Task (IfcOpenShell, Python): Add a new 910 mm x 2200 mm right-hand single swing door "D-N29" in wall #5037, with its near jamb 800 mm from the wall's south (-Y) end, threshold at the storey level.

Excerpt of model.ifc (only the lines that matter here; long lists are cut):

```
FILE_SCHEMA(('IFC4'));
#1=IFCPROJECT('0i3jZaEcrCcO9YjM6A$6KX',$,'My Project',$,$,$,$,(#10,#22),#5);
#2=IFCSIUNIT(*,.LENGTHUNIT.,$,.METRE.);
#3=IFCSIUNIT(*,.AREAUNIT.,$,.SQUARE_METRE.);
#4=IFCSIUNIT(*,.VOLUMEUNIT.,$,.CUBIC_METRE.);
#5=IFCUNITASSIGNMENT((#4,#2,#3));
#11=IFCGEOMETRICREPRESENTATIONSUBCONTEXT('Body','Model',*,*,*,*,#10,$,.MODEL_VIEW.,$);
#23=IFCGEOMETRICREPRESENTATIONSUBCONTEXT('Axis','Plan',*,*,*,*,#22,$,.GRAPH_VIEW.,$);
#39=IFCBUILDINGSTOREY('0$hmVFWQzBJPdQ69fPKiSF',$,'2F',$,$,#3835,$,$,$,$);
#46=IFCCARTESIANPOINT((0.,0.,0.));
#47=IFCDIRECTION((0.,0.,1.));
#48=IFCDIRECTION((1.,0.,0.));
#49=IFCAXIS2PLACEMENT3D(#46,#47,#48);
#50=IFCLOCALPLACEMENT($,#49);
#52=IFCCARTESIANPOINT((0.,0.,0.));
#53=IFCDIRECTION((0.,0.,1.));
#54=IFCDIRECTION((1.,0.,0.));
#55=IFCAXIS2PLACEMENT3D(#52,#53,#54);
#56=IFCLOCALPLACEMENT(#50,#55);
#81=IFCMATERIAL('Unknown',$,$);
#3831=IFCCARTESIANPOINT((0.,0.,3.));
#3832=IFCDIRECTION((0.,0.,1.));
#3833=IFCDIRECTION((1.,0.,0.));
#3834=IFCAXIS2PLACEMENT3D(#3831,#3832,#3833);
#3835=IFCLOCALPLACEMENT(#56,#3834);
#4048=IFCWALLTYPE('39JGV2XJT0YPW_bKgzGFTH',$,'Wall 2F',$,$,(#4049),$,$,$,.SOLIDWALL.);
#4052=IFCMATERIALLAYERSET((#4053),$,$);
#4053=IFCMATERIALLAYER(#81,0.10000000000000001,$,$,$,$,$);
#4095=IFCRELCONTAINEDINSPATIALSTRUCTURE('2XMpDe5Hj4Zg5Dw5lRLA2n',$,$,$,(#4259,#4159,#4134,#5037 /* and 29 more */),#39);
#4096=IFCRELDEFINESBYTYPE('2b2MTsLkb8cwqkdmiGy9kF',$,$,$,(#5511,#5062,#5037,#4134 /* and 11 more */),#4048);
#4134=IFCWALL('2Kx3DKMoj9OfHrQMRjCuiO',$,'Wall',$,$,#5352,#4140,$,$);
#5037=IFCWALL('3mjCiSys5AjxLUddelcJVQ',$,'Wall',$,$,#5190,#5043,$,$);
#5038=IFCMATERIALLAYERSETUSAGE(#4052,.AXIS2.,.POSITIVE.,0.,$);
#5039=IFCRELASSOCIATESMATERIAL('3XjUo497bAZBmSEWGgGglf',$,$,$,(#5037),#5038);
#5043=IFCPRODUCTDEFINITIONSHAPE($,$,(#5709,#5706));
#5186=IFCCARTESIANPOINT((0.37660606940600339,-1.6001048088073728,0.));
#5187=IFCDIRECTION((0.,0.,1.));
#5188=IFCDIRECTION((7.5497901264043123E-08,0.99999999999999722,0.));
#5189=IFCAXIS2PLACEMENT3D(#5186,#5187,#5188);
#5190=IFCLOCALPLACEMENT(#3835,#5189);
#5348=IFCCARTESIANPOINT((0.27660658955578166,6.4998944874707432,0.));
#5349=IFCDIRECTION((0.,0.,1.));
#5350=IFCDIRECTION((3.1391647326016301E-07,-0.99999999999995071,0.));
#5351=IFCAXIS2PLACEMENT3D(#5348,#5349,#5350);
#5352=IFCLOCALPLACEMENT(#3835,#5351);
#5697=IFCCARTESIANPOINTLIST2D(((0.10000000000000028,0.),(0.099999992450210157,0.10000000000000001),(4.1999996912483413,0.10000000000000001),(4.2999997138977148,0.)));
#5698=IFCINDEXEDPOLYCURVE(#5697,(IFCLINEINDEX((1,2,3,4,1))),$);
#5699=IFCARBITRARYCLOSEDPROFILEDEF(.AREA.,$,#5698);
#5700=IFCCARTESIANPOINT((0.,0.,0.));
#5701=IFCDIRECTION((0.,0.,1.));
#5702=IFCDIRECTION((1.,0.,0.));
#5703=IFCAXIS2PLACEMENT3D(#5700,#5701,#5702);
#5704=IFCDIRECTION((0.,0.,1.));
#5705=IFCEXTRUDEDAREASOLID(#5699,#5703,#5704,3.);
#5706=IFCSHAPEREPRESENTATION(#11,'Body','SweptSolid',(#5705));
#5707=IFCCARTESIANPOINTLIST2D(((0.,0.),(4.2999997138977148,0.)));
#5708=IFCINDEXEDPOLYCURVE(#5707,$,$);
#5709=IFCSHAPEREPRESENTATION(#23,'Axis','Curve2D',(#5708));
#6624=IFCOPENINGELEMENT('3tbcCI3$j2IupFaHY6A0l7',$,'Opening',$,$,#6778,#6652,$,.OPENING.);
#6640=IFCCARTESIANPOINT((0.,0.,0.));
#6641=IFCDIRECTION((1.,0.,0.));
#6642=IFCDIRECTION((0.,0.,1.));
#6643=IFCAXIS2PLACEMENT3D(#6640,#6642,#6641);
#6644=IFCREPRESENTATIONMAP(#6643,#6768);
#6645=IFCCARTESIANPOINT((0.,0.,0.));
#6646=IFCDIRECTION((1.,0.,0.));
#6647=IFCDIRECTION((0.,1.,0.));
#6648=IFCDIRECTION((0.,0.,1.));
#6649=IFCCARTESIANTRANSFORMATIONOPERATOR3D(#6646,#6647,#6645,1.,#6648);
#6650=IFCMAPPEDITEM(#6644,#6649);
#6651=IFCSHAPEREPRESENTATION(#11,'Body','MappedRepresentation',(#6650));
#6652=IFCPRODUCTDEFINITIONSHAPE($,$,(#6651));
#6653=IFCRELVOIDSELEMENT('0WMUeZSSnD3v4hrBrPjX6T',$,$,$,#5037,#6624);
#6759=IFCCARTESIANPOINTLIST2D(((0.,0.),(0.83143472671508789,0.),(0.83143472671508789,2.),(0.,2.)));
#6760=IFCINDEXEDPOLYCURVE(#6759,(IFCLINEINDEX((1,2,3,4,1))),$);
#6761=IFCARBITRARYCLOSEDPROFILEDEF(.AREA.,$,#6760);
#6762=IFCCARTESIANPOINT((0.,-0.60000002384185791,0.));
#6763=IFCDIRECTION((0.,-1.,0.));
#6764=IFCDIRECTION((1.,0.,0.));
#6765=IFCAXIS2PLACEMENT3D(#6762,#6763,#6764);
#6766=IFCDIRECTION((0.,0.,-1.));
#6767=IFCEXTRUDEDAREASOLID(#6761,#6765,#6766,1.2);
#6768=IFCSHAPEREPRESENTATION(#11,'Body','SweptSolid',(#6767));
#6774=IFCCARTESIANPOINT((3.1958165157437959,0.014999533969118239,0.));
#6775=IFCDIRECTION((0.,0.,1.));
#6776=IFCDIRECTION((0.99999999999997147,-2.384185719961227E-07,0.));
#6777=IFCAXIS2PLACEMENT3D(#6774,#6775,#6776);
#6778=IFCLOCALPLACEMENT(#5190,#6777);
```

```python
import numpy as np
import ifcopenshell
import ifcopenshell.api.feature
import ifcopenshell.api.geometry
import ifcopenshell.api.root
import ifcopenshell.api.spatial
import ifcopenshell.geom
import ifcopenshell.util.element
import ifcopenshell.util.placement
import ifcopenshell.util.representation
import ifcopenshell.util.shape
import ifcopenshell.util.unit

model = ifcopenshell.open("model.ifc")
unit_scale = ifcopenshell.util.unit.calculate_unit_scale(model)
settings = ifcopenshell.geom.settings()


def volume(element):
    """Net volume in cubic metres, openings subtracted."""
    shape = ifcopenshell.geom.create_shape(settings, element)
    return ifcopenshell.util.shape.get_volume(shape.geometry)


wall = model.by_guid("3mjCiSys5AjxLUddelcJVQ")
storey = ifcopenshell.util.element.get_container(wall, ifc_class="IfcBuildingStorey")
context = ifcopenshell.util.representation.get_context(model, "Model", "Body", "MODEL_VIEW")
before = volume(wall)

width, height, from_end, sill = 0.91, 2.2, 0.8, 0.0  # metres

# The wall runs along its own X axis, and the end named is its -X end.
wall_shape = ifcopenshell.geom.create_shape(settings, wall)
x, y, z = ifcopenshell.util.shape.get_vertices(wall_shape.geometry).T
start = x.min() + from_end
face, thickness = float(y.min()), float(y.max() - y.min())
wall_matrix = ifcopenshell.util.placement.get_local_placement(wall.ObjectPlacement)
level = ifcopenshell.util.placement.get_local_placement(storey.ObjectPlacement)[2, 3]


def in_wall(x, y):
    """Placement at x, y metres in the wall's axes, at sill height."""
    matrix = wall_matrix.copy()
    matrix[:, 3] = wall_matrix @ np.array([x / unit_scale, y / unit_scale, 0.0, 1.0])
    matrix[2, 3] = level + sill / unit_scale
    return matrix


# Opening: a box that overshoots both wall faces by 50 mm.
opening = ifcopenshell.api.root.create_entity(model, ifc_class="IfcOpeningElement", predefined_type="OPENING")
box = ifcopenshell.api.geometry.add_wall_representation(
    model, context=context, length=width, height=height, thickness=thickness + 0.1
)
ifcopenshell.api.geometry.assign_representation(model, product=opening, representation=box)
ifcopenshell.api.geometry.edit_object_placement(model, product=opening, matrix=in_wall(start, face - 0.05), is_si=False)
ifcopenshell.api.feature.add_feature(model, feature=opening, element=wall)

door = ifcopenshell.api.root.create_entity(model, ifc_class="IfcDoor", name="D-N29", predefined_type="DOOR")
door.OverallWidth, door.OverallHeight = width / unit_scale, height / unit_scale
door.OperationType = "SINGLE_SWING_RIGHT"
body = ifcopenshell.api.geometry.add_door_representation(
    model,
    context=context,
    overall_width=door.OverallWidth,
    overall_height=door.OverallHeight,
    operation_type="SINGLE_SWING_RIGHT",
    lining_properties={"LiningDepth": thickness / unit_scale, "ThresholdDepth": thickness / unit_scale},
)
ifcopenshell.api.geometry.assign_representation(model, product=door, representation=body)
ifcopenshell.api.spatial.assign_container(model, products=[door], relating_structure=storey)
ifcopenshell.api.feature.add_filling(model, opening=opening, element=door)

# The lining spans the wall, so the door starts at the wall face.
ifcopenshell.api.geometry.edit_object_placement(model, product=door, matrix=in_wall(start, face), is_si=False)

after = volume(wall)

print(f"wall volume {before:.3f} -> {after:.3f} m3")

model.write("model_edited.ifc")
```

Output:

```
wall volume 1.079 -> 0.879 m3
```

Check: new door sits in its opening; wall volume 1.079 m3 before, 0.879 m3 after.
